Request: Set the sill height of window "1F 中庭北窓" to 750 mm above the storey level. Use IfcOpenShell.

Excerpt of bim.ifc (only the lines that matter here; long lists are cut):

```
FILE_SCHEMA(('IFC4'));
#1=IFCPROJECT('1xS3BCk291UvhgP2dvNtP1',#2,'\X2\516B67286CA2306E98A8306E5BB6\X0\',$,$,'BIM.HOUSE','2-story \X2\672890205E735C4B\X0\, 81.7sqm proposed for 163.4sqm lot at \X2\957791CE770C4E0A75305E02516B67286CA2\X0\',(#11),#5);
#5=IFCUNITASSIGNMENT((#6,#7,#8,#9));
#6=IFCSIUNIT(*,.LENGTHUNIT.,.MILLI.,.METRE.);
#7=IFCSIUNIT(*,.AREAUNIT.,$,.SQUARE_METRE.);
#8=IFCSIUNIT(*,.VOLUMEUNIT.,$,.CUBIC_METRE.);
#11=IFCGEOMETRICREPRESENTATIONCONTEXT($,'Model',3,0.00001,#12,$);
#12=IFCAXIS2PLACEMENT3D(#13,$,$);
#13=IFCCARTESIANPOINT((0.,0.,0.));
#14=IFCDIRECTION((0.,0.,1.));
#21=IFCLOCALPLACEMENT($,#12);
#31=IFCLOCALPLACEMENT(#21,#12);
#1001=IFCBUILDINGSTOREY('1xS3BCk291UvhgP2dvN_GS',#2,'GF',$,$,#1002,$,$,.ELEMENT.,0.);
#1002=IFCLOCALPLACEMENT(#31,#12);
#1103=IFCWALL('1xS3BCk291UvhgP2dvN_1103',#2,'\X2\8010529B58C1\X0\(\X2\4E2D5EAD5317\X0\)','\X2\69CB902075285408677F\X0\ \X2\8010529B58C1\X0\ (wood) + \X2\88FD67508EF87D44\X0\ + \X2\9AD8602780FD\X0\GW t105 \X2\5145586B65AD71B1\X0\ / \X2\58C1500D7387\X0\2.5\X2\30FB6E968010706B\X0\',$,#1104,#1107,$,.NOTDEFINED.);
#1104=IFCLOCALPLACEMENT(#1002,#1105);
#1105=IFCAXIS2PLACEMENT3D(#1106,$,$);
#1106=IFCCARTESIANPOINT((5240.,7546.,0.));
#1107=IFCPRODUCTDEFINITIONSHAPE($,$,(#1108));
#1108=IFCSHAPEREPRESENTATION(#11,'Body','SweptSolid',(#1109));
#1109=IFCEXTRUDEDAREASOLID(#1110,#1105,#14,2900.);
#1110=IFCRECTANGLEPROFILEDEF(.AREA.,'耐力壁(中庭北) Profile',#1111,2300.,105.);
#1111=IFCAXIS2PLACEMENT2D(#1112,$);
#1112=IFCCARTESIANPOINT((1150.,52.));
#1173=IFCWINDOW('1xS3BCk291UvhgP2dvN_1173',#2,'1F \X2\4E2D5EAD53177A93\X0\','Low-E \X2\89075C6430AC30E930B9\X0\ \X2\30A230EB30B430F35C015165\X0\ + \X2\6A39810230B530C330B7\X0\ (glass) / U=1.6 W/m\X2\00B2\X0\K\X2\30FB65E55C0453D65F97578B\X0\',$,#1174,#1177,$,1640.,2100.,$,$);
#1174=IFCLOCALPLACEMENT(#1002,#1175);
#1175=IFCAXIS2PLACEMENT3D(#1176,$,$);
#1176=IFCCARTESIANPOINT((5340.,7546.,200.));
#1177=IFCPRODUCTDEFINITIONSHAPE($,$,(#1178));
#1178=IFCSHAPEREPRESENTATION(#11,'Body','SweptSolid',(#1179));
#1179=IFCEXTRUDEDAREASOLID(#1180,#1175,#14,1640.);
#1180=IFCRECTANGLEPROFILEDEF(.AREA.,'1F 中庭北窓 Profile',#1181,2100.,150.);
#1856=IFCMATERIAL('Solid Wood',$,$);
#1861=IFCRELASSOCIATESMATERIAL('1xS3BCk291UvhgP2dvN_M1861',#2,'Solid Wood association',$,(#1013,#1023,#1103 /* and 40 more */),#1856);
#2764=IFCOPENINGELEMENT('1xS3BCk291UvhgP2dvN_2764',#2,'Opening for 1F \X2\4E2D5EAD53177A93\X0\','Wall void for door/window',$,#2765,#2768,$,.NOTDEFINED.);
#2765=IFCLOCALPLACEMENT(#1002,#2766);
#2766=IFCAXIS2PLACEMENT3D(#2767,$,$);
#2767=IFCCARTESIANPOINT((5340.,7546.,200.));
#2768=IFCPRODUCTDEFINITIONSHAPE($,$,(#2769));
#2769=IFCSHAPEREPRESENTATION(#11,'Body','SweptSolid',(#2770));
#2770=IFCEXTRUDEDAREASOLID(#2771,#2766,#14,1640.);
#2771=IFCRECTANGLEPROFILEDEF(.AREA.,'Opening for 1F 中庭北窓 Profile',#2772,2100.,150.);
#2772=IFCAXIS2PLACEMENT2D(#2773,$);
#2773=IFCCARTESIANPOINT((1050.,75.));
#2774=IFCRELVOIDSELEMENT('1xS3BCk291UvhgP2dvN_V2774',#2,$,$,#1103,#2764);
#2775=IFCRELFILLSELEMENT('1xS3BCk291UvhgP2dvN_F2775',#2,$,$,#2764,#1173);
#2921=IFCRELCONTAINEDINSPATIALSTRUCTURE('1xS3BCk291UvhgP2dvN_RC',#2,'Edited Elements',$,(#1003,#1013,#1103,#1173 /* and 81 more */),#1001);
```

```python
import numpy as np
import ifcopenshell
import ifcopenshell.api.geometry
import ifcopenshell.geom
import ifcopenshell.util.element
import ifcopenshell.util.placement
import ifcopenshell.util.shape
import ifcopenshell.util.unit

model = ifcopenshell.open("bim.ifc")
unit_scale = ifcopenshell.util.unit.calculate_unit_scale(model)

window = model.by_guid("1xS3BCk291UvhgP2dvN_1173")
opening = window.FillsVoids[0].RelatingOpeningElement
storey = ifcopenshell.util.element.get_container(window, ifc_class="IfcBuildingStorey")
level = ifcopenshell.util.placement.get_local_placement(storey.ObjectPlacement)[2, 3]

# The opening's origin need not be at the sill, so measure its lowest point.
shape = ifcopenshell.geom.create_shape(ifcopenshell.geom.settings(), opening)
bottom = ifcopenshell.util.shape.get_shape_bottom_elevation(shape, shape.geometry) / unit_scale
dz = level + 750.0 - bottom

shift = np.array([0.0, 0.0, dz])
# The window is not placed relative to its opening, so move both.
for product in (opening, window):
    matrix = ifcopenshell.util.placement.get_local_placement(product.ObjectPlacement)
    matrix[:3, 3] += shift
    ifcopenshell.api.geometry.edit_object_placement(model, product=product, matrix=matrix, is_si=False)

print(f"moved by {dz * unit_scale:+.3f} m")

model.write("bim_v2.ifc")
```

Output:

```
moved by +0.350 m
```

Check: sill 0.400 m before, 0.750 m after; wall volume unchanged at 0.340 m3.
